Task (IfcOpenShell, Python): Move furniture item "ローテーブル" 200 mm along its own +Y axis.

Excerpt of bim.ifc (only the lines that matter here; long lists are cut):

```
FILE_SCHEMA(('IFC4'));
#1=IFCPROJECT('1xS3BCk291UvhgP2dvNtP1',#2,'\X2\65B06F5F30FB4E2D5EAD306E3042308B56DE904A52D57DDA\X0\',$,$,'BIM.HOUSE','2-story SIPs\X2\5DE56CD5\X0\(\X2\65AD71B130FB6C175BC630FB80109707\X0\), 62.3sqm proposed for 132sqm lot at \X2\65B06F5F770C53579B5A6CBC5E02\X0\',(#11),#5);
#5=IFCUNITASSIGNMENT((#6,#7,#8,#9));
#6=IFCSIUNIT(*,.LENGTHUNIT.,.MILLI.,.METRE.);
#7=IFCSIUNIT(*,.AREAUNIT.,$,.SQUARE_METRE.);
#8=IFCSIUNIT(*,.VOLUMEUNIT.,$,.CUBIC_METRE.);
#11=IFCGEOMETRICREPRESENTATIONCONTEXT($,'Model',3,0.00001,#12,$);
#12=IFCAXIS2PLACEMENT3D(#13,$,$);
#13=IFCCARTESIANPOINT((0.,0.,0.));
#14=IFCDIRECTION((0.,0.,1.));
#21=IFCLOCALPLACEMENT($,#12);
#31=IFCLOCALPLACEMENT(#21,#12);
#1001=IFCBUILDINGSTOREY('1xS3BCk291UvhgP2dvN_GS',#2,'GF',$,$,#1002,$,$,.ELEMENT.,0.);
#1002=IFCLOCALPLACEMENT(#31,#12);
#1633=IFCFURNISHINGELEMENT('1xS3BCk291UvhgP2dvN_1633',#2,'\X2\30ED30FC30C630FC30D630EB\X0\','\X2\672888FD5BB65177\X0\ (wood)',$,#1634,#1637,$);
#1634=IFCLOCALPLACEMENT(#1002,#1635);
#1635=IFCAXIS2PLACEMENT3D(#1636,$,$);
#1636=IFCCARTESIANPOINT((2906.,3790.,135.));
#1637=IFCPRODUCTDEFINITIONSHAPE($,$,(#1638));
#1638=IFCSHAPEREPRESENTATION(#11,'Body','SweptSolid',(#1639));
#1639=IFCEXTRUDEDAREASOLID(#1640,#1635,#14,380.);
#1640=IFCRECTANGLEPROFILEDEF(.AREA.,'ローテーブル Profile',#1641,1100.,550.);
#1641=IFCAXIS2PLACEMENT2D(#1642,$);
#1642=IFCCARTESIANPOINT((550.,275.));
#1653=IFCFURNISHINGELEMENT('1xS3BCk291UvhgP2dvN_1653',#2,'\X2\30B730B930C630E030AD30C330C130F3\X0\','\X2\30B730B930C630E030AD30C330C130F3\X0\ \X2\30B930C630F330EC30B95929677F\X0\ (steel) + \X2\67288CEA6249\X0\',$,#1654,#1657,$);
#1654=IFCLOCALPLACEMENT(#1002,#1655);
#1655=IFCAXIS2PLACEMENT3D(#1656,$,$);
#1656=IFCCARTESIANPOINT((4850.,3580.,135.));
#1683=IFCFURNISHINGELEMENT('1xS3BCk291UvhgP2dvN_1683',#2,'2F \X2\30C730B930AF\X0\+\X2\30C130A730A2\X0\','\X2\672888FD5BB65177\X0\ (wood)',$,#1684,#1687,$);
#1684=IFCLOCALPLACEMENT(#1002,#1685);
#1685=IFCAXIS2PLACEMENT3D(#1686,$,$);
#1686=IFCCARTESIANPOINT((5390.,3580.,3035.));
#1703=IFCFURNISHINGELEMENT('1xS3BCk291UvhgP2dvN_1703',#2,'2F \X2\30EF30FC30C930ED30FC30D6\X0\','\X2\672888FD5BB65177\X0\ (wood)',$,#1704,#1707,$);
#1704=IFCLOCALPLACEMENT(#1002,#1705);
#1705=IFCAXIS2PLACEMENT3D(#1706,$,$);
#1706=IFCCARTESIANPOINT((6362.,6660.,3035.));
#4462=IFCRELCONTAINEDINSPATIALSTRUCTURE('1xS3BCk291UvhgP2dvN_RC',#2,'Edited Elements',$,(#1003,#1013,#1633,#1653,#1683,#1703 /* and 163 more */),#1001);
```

```python
import ifcopenshell
import ifcopenshell.api.geometry
import ifcopenshell.util.placement
import ifcopenshell.util.unit

model = ifcopenshell.open("bim.ifc")
unit_scale = ifcopenshell.util.unit.calculate_unit_scale(model)

item = model.by_guid("1xS3BCk291UvhgP2dvN_1633")
matrix = ifcopenshell.util.placement.get_local_placement(item.ObjectPlacement)
matrix[:3, 3] += matrix[:3, 1] * 0.2 / unit_scale
ifcopenshell.api.geometry.edit_object_placement(model, product=item, matrix=matrix, is_si=False)

print(ifcopenshell.util.placement.get_local_placement(item.ObjectPlacement).round(3) + 0.0)

model.write("bim_updated.ifc")
```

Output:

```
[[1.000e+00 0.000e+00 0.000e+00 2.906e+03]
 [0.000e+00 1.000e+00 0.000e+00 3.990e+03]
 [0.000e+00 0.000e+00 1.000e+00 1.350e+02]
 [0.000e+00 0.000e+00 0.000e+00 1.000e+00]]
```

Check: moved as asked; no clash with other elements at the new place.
